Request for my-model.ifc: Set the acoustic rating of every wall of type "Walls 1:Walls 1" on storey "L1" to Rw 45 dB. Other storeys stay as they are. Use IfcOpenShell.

First a look at what the model holds.

```python
import ifcopenshell
import ifcopenshell.util.element

model = ifcopenshell.open("my-model.ifc")
print(model.schema)
storey = next(s for s in model.by_type("IfcBuildingStorey") if s.Name == "L1")
walls = [e for e in ifcopenshell.util.element.get_decomposition(storey) if e.is_a("IfcWall")]
seen = {}
for e in walls:
    element_type = ifcopenshell.util.element.get_type(e)
    key = (element_type.Name if element_type != e and element_type else None, ifcopenshell.util.element.get_pset(e, "Pset_WallCommon", "AcousticRating"))
    seen[key] = seen.get(key, 0) + 1
for (name, value), count in sorted(seen.items(), key=str):
    print(count, "x", name, "|", value)
```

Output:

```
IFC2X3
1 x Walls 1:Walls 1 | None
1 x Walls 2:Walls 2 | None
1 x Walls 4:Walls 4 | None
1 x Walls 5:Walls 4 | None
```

```python
import ifcopenshell
import ifcopenshell.api.pset
import ifcopenshell.util.element

model = ifcopenshell.open("my-model.ifc")

storey = next(s for s in model.by_type("IfcBuildingStorey") if s.Name == "L1")
walls = [e for e in ifcopenshell.util.element.get_decomposition(storey) if e.is_a("IfcWall")]

count = 0
for e in walls:
    element_type = ifcopenshell.util.element.get_type(e)
    if element_type in (None, e) or element_type.Name != "Walls 1:Walls 1":
        continue
    # add_pset returns the element's existing set when there is one.
    pset = ifcopenshell.api.pset.add_pset(model, product=e, name="Pset_WallCommon")
    ifcopenshell.api.pset.edit_pset(model, pset=pset, properties={"AcousticRating": "Rw 45 dB"})
    count += 1

print(count, "walls updated")

model.write("my-model_updated.ifc")
```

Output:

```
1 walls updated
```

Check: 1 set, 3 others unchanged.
